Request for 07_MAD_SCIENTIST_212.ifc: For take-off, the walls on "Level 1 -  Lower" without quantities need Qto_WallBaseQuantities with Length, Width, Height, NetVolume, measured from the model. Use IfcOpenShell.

First a look at what the model holds.

```python
import ifcopenshell
import ifcopenshell.util.element
import ifcopenshell.util.unit

model = ifcopenshell.open("07_MAD_SCIENTIST_212.ifc")
print(model.schema)
for unit_type in ("LENGTHUNIT", "AREAUNIT", "VOLUMEUNIT"):
    print(unit_type, ifcopenshell.util.unit.calculate_unit_scale(model, unit_type))
storey = next(s for s in model.by_type("IfcBuildingStorey") if s.Name == "Level 1 -  Lower")
walls = [e for e in ifcopenshell.util.element.get_decomposition(storey) if e.is_a("IfcWall")]
for e in sorted(walls, key=lambda e: e.id()):
    print(e.id(), e.is_a(), e.Name, list(ifcopenshell.util.element.get_psets(e, qtos_only=True)), sep=" | ")
```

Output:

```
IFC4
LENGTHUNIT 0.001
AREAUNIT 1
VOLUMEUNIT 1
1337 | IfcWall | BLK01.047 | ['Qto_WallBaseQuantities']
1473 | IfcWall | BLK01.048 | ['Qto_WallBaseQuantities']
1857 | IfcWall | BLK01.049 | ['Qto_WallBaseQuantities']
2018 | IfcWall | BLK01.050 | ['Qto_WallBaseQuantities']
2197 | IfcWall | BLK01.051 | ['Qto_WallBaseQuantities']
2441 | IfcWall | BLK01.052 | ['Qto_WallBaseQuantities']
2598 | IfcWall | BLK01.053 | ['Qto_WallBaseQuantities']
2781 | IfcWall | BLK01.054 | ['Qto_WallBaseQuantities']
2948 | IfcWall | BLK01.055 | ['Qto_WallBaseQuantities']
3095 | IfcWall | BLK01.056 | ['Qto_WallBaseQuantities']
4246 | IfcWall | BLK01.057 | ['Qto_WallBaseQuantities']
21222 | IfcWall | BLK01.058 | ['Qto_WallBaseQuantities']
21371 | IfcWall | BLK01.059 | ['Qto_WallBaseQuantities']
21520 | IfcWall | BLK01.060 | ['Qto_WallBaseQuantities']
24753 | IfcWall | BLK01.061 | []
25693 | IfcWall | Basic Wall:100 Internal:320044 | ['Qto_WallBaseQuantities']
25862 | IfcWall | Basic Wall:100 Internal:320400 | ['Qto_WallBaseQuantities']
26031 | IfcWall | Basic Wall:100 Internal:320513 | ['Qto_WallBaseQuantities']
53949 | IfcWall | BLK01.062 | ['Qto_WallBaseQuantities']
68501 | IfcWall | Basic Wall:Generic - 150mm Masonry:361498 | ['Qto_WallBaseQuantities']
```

```python
import ifcopenshell
import ifcopenshell.api.pset
import ifcopenshell.geom
import ifcopenshell.util.element
import ifcopenshell.util.shape
import ifcopenshell.util.unit

model = ifcopenshell.open("07_MAD_SCIENTIST_212.ifc")
unit_scale = ifcopenshell.util.unit.calculate_unit_scale(model)
volume_scale = ifcopenshell.util.unit.calculate_unit_scale(model, "VOLUMEUNIT")
settings = ifcopenshell.geom.settings()

storey = next(s for s in model.by_type("IfcBuildingStorey") if s.Name == "Level 1 -  Lower")
walls = [e for e in ifcopenshell.util.element.get_decomposition(storey) if e.is_a("IfcWall")]

for e in sorted(walls, key=lambda e: e.id()):
    if ifcopenshell.util.element.get_psets(e, qtos_only=True, should_inherit=False):
        continue
    # Geometry comes back in metres, in the element's own axes.
    shape = ifcopenshell.geom.create_shape(settings, e)
    values = {
        "Length": ifcopenshell.util.shape.get_x(shape.geometry) / unit_scale,
        "Width": ifcopenshell.util.shape.get_y(shape.geometry) / unit_scale,
        "Height": ifcopenshell.util.shape.get_z(shape.geometry) / unit_scale,
        "NetVolume": ifcopenshell.util.shape.get_volume(shape.geometry) / volume_scale,
    }
    qto = ifcopenshell.api.pset.add_qto(model, product=e, name="Qto_WallBaseQuantities")
    ifcopenshell.api.pset.edit_qto(model, qto=qto, properties=values)
    print(e.id(), {k: round(v, 3) for k, v in values.items()})

model.write("07_MAD_SCIENTIST_212_edited.ifc")
```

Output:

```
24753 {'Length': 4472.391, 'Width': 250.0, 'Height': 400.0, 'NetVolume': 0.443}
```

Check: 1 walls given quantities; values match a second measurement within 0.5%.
